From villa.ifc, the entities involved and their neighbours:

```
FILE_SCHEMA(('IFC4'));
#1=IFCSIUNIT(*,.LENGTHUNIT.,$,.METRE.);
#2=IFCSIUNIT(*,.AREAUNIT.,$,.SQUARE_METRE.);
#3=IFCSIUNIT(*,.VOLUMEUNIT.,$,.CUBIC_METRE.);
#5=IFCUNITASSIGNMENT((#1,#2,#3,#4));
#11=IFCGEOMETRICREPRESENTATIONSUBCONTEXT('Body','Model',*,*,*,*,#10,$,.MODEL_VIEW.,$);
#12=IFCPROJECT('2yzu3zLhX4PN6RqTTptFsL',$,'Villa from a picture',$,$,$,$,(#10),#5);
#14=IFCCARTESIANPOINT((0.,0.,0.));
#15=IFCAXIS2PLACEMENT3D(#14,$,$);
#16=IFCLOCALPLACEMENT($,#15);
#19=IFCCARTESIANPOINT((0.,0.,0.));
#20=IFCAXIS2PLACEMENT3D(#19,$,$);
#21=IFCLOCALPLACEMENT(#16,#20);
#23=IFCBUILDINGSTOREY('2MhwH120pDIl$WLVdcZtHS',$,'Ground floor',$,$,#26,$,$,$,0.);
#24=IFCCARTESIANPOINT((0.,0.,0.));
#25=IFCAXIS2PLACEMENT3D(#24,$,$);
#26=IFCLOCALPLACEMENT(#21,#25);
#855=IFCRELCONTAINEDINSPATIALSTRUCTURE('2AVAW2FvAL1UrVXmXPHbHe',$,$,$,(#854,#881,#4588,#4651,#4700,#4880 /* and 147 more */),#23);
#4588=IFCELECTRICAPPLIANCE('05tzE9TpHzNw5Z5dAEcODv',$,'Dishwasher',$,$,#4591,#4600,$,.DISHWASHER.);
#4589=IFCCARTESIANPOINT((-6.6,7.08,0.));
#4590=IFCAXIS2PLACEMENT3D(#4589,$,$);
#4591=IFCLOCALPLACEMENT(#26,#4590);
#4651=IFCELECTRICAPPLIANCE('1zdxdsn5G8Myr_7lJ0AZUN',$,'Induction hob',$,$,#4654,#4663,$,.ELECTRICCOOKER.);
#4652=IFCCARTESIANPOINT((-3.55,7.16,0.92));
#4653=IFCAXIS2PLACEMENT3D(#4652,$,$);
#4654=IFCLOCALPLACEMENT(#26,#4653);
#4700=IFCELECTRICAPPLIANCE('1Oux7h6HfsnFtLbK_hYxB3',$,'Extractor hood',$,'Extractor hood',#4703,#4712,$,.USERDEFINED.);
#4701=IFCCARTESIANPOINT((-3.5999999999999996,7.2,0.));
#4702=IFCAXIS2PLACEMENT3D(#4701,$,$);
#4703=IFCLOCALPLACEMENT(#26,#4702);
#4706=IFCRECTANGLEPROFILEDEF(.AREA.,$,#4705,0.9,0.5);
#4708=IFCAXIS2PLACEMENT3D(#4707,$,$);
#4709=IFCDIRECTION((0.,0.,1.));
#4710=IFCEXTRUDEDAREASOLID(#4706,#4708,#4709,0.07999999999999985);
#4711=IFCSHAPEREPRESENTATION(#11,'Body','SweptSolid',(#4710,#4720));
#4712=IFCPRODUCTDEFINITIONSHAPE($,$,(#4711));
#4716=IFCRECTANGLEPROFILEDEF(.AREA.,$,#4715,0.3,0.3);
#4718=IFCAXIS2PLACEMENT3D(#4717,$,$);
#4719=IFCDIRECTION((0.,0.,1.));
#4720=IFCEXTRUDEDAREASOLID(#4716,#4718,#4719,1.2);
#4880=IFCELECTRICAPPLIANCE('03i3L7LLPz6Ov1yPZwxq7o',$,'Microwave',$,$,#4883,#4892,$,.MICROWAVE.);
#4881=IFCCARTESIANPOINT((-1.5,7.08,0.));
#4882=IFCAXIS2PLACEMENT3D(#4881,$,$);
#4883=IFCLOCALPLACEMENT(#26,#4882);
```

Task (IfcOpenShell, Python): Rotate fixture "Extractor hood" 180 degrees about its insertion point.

```python
import ifcopenshell
import ifcopenshell.api.geometry
import ifcopenshell.util.placement

model = ifcopenshell.open("villa.ifc")

item = model.by_guid("1Oux7h6HfsnFtLbK_hYxB3")
matrix = ifcopenshell.util.placement.get_local_placement(item.ObjectPlacement)
matrix = matrix @ ifcopenshell.util.placement.rotation(180, "Z")
ifcopenshell.api.geometry.edit_object_placement(model, product=item, matrix=matrix, is_si=False)

print(ifcopenshell.util.placement.get_local_placement(item.ObjectPlacement).round(3) + 0.0)

model.write("villa_v2.ifc")
```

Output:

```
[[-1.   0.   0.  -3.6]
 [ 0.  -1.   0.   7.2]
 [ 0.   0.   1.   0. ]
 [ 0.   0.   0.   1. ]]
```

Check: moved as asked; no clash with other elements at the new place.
